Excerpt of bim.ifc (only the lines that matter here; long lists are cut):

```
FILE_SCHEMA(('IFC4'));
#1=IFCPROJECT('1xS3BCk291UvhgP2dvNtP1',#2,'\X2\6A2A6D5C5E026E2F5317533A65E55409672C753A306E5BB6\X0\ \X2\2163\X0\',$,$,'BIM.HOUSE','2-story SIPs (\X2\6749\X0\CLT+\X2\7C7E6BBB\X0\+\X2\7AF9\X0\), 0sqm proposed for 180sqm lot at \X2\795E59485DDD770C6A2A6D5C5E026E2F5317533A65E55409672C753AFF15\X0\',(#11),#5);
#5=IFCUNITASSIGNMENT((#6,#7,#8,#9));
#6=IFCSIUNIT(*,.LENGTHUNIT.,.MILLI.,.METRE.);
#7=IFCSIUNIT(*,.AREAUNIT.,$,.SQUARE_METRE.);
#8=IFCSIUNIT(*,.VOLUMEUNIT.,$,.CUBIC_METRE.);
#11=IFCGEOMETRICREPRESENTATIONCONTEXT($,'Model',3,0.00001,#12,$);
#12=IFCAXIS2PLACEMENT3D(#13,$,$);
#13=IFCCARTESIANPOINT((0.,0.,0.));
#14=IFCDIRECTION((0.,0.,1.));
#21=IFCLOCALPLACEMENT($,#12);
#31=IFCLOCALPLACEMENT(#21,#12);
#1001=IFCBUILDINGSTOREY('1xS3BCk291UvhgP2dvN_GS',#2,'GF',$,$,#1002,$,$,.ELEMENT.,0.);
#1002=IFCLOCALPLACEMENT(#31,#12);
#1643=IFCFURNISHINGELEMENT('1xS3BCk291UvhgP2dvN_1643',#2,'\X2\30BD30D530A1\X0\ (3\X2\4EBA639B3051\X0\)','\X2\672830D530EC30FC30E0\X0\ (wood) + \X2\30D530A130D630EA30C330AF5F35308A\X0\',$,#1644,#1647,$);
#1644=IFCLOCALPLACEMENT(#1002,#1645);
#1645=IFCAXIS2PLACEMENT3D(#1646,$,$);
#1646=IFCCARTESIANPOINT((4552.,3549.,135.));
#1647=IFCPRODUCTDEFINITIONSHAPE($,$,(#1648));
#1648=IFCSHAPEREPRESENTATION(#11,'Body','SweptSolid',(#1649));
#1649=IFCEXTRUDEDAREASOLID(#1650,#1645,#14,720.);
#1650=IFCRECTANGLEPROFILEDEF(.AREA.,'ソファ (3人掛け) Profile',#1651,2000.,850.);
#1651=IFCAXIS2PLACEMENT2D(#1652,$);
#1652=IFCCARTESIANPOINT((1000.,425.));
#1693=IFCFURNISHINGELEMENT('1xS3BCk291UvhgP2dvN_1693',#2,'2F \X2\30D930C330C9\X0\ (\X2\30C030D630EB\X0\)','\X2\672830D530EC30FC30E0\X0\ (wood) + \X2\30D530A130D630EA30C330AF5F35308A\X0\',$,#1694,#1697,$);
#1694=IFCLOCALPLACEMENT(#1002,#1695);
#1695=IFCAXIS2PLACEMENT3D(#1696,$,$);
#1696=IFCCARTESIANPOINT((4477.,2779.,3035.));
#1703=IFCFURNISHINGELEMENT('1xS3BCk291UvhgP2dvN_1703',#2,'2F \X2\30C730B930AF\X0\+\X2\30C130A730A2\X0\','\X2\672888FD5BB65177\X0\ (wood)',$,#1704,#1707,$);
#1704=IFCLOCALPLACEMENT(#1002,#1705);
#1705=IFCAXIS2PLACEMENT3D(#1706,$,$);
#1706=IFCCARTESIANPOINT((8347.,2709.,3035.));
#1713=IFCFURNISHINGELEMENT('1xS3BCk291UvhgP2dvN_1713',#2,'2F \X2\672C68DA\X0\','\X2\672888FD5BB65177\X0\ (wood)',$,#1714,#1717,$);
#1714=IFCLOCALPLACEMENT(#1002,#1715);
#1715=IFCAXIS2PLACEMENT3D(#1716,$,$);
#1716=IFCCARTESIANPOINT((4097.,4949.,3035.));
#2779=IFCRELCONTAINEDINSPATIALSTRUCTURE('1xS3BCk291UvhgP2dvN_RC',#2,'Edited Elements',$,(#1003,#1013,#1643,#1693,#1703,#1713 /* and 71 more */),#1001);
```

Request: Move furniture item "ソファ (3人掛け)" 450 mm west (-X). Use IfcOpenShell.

```python
import ifcopenshell
import ifcopenshell.api.geometry
import ifcopenshell.util.placement
import ifcopenshell.util.unit

model = ifcopenshell.open("bim.ifc")
unit_scale = ifcopenshell.util.unit.calculate_unit_scale(model)

item = model.by_guid("1xS3BCk291UvhgP2dvN_1643")
matrix = ifcopenshell.util.placement.get_local_placement(item.ObjectPlacement)
matrix[0, 3] -= 0.45 / unit_scale
ifcopenshell.api.geometry.edit_object_placement(model, product=item, matrix=matrix, is_si=False)

print(ifcopenshell.util.placement.get_local_placement(item.ObjectPlacement).round(3) + 0.0)

model.write("bim-out.ifc")
```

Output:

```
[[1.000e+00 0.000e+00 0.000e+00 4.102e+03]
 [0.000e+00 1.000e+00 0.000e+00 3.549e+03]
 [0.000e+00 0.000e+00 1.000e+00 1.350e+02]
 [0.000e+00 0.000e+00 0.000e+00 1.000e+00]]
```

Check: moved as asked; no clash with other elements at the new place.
